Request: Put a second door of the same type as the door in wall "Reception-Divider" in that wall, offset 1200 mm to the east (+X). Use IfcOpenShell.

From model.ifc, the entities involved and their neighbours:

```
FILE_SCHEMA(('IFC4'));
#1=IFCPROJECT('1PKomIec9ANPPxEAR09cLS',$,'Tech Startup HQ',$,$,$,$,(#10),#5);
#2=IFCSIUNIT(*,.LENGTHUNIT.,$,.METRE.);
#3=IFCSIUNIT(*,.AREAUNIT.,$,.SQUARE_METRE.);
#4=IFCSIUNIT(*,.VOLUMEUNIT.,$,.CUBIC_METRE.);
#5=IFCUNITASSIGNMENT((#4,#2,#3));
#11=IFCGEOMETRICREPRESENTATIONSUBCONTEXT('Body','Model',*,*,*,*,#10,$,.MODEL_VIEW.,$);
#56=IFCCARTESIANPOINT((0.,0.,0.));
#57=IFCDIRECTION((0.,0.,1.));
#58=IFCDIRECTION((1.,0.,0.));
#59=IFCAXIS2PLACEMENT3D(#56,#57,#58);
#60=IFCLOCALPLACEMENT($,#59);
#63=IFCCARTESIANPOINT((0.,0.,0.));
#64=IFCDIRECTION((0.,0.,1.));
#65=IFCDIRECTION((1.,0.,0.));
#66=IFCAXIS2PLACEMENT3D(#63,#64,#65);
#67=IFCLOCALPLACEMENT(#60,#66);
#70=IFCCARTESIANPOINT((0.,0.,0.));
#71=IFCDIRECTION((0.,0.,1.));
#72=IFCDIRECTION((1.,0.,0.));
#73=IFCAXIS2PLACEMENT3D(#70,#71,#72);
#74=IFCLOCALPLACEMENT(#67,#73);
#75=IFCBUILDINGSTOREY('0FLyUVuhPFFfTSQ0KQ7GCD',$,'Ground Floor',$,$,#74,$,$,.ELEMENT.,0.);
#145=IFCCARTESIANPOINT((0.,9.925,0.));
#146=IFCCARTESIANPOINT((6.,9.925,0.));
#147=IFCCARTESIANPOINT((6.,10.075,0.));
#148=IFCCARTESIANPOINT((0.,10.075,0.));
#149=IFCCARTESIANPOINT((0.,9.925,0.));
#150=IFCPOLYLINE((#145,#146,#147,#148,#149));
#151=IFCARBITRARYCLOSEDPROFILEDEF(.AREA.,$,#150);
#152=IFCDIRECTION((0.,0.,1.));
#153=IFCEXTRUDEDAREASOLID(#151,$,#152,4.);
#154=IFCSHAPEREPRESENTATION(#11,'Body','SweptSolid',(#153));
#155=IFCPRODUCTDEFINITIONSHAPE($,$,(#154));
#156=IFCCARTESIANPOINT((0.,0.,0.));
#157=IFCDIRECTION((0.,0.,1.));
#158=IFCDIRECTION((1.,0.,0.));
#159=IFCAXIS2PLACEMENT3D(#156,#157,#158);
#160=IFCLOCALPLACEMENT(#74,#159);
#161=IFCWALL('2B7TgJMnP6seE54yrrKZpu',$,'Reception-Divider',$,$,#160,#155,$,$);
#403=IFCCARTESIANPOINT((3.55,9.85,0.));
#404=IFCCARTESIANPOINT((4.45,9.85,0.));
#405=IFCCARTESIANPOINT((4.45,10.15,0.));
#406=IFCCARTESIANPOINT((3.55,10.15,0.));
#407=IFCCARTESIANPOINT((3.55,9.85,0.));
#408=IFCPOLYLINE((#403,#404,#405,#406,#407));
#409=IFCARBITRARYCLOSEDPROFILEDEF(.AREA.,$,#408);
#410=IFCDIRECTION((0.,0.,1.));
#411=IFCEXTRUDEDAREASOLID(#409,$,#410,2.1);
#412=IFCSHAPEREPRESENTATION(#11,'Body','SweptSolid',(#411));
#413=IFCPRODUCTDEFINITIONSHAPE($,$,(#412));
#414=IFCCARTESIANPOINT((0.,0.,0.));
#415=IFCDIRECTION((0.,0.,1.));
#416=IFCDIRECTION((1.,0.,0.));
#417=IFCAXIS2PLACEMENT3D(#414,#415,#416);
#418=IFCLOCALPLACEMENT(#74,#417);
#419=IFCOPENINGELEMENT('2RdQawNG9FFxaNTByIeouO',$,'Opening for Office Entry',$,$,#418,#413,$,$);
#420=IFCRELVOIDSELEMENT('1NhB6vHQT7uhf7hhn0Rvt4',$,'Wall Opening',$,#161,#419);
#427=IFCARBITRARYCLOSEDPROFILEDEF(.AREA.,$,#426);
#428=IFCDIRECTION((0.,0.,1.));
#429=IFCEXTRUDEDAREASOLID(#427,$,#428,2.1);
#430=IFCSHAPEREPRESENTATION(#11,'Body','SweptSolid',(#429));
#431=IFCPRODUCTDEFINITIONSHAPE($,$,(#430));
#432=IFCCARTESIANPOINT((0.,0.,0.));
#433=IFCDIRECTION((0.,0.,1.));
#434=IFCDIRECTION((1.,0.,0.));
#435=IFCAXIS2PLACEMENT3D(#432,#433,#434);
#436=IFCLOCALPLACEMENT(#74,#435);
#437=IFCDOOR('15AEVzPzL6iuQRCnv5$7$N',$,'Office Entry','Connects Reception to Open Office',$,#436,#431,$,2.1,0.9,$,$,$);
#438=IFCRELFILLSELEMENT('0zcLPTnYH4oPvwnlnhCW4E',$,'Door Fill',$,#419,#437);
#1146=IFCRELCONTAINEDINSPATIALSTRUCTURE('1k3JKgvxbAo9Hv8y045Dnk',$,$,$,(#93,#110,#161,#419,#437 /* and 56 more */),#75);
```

```python
import ifcopenshell
import ifcopenshell.api.feature
import ifcopenshell.api.geometry
import ifcopenshell.api.root
import ifcopenshell.geom
import ifcopenshell.util.element
import ifcopenshell.util.placement
import ifcopenshell.util.shape
import ifcopenshell.util.unit

model = ifcopenshell.open("model.ifc")
unit_scale = ifcopenshell.util.unit.calculate_unit_scale(model)
settings = ifcopenshell.geom.settings()


def volume(element):
    """Net volume in cubic metres, openings subtracted."""
    shape = ifcopenshell.geom.create_shape(settings, element)
    return ifcopenshell.util.shape.get_volume(shape.geometry)


door = model.by_guid("15AEVzPzL6iuQRCnv5$7$N")
opening = door.FillsVoids[0].RelatingOpeningElement
wall = opening.VoidsElements[0].RelatingBuildingElement
before = volume(wall)
shift = ifcopenshell.util.placement.get_local_placement(wall.ObjectPlacement)[:3, 0] * 1.2 / unit_scale

# copy_class copies the void relationship, type, container and properties, but no geometry.
new_opening = ifcopenshell.api.root.copy_class(model, product=opening)
new_opening.Representation = ifcopenshell.util.element.copy_deep(
    model, opening.Representation, exclude=["IfcGeometricRepresentationContext", "IfcRepresentationMap"]
)
new_door = ifcopenshell.api.root.copy_class(model, product=door)
new_door.Representation = ifcopenshell.util.element.copy_deep(
    model, door.Representation, exclude=["IfcGeometricRepresentationContext", "IfcRepresentationMap"]
)
ifcopenshell.api.feature.add_filling(model, opening=new_opening, element=new_door)

for old, new in ((opening, new_opening), (door, new_door)):
    matrix = ifcopenshell.util.placement.get_local_placement(old.ObjectPlacement)
    matrix[:3, 3] += shift
    ifcopenshell.api.geometry.edit_object_placement(model, product=new, matrix=matrix, is_si=False)

after = volume(wall)

print(f"wall volume {before:.3f} -> {after:.3f} m3")

model.write("model_v2.ifc")
```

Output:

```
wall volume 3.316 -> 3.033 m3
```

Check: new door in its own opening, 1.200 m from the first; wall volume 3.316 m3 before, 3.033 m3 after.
